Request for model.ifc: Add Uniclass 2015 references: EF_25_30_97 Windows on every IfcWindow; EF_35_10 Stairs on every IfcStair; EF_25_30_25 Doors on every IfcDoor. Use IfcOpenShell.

First a look at what the model holds.

```python
import ifcopenshell

model = ifcopenshell.open("model.ifc")
print(model.schema)
print("classifications:", [c.Name for c in model.by_type("IfcClassification")])
for ifc_class in ("IfcDoor", "IfcRoof", "IfcStair", "IfcWall", "IfcWindow"):
    print(ifc_class, len(model.by_type(ifc_class)))
```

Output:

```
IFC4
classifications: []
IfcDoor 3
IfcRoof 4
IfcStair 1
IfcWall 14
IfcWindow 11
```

```python
import ifcopenshell
import ifcopenshell.api.classification

model = ifcopenshell.open("model.ifc")

system = ifcopenshell.api.classification.add_classification(model, classification="Uniclass 2015")

codes = {
    "IfcWindow": ("EF_25_30_97", "Windows"),
    "IfcStair": ("EF_35_10", "Stairs"),
    "IfcDoor": ("EF_25_30_25", "Doors"),
}
for ifc_class, (code, name) in codes.items():
    products = model.by_type(ifc_class)
    ifcopenshell.api.classification.add_reference(
        model, products=products, classification=system, identification=code, name=name
    )
    print(code, len(products))

model.write("model_updated.ifc")
```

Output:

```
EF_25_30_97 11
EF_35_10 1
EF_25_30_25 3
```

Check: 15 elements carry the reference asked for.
